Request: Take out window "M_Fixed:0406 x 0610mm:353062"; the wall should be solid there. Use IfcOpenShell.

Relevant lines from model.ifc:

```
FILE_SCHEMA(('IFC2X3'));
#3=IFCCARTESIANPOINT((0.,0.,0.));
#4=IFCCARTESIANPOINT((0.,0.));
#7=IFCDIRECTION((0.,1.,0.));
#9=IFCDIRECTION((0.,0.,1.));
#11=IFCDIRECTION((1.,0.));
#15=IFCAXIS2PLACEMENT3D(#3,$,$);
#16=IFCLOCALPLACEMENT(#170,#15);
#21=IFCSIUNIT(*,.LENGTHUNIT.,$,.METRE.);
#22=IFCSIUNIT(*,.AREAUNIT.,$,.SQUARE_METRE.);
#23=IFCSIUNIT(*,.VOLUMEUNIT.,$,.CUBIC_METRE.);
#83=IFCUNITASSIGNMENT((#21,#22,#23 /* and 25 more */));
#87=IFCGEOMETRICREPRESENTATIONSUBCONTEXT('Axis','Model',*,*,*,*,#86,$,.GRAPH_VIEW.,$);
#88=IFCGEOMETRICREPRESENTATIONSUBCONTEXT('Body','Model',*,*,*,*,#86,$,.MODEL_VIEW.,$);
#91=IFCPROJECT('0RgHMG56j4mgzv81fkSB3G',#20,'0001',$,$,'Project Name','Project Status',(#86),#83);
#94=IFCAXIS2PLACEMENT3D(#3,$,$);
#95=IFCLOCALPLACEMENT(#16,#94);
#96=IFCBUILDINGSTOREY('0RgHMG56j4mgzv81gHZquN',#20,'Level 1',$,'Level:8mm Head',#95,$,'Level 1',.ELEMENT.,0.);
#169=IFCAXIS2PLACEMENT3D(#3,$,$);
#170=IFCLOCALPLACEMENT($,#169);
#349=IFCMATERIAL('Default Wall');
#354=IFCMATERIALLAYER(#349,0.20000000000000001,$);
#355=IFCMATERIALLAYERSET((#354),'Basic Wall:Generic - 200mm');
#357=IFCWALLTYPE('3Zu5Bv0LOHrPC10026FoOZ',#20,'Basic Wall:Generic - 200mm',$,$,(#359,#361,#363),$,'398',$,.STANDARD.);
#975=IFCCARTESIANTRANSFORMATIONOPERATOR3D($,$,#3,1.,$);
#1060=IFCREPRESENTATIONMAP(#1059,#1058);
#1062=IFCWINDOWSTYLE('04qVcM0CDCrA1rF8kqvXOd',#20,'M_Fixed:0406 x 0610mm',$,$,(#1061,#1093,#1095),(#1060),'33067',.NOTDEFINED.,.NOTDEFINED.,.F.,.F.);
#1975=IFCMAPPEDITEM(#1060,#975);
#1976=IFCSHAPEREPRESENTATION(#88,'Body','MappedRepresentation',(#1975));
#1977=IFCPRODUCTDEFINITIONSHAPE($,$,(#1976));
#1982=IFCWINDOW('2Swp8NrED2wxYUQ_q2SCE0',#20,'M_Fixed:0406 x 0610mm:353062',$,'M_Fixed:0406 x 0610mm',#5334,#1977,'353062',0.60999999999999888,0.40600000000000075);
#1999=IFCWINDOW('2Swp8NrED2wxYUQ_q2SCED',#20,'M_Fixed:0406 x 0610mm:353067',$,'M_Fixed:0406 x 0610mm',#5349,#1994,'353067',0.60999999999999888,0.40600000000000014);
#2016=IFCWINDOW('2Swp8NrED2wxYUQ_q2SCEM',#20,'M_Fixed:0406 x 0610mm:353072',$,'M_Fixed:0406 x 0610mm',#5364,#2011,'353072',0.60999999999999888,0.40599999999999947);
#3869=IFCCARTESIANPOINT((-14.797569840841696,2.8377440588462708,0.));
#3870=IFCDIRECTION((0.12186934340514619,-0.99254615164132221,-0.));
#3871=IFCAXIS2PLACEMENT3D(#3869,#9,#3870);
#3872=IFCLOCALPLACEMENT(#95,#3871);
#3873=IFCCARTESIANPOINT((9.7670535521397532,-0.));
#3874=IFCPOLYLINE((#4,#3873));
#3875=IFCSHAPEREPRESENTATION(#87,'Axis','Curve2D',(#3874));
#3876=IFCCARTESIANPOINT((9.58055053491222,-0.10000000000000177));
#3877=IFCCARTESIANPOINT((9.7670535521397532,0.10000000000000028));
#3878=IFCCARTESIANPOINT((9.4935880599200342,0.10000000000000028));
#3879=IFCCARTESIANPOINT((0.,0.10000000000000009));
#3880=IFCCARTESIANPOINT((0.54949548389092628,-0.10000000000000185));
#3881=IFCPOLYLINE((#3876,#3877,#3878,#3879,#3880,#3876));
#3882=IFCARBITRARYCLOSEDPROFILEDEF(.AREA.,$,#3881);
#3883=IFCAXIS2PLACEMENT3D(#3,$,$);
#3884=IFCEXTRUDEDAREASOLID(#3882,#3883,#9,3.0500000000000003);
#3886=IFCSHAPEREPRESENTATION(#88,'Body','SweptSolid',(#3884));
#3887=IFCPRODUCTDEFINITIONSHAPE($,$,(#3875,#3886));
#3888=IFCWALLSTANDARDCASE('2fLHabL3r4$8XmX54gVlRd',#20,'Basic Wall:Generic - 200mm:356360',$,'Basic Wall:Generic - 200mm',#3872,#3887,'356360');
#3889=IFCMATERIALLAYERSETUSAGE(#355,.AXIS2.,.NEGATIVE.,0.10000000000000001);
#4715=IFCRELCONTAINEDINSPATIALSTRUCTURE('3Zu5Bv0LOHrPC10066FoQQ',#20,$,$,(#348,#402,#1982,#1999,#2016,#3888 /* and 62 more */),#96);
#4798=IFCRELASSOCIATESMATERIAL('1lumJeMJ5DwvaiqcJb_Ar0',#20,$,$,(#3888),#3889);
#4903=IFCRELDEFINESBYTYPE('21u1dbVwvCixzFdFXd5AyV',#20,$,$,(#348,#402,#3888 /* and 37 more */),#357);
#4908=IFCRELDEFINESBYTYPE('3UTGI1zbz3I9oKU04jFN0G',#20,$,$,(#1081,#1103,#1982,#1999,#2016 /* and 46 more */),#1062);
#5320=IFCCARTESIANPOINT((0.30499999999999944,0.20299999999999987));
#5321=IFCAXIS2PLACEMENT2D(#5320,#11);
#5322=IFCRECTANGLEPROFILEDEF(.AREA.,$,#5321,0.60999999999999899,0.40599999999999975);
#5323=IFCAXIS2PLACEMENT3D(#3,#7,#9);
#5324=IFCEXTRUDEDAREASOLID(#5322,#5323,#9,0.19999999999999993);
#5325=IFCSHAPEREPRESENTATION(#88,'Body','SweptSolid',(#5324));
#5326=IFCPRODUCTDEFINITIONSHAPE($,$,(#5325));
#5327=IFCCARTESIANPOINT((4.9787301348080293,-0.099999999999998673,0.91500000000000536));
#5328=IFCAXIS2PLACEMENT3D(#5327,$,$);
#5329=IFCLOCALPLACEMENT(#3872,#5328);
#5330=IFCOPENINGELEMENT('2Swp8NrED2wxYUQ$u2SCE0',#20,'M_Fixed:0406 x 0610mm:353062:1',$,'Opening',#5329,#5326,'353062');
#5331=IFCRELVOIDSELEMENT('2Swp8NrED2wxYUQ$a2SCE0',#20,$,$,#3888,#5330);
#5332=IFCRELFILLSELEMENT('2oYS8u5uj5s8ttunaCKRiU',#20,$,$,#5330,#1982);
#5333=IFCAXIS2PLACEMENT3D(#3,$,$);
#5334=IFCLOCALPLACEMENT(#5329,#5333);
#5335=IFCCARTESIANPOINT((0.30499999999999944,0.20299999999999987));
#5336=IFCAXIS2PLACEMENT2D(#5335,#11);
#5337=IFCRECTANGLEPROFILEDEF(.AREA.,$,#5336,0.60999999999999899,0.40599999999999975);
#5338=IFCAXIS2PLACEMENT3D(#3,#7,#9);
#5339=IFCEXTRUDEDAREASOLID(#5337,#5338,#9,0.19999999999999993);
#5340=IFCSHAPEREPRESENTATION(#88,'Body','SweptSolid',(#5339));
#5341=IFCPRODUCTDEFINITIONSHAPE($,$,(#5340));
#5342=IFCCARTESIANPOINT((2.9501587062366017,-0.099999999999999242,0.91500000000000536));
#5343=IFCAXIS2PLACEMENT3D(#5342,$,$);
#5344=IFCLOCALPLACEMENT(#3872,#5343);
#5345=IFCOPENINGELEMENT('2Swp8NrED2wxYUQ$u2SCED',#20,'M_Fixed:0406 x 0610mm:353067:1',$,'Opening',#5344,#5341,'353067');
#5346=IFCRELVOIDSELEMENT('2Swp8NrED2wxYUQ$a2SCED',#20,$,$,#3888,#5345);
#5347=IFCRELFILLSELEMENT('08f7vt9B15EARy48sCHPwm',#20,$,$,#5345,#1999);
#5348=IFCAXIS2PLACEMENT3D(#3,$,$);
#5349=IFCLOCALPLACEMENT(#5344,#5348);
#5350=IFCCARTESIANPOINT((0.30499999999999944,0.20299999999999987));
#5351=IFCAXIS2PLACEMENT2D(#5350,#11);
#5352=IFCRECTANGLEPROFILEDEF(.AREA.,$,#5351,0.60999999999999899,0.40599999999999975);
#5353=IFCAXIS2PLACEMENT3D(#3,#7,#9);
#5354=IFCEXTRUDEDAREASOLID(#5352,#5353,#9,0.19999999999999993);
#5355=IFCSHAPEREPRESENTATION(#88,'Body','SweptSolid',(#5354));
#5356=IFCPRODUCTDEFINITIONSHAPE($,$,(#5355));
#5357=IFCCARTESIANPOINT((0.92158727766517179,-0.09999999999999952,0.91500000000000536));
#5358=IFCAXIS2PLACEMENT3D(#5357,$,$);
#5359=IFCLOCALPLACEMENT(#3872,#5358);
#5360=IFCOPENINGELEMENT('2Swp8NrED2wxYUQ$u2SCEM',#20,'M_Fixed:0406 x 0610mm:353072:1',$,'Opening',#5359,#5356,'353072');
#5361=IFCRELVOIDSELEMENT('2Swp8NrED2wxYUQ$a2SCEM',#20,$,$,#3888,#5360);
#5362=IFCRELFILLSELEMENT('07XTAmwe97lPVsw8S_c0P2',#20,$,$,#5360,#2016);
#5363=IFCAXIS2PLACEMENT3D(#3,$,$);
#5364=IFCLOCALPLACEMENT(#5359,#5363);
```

```python
import ifcopenshell
import ifcopenshell.api.feature
import ifcopenshell.api.root
import ifcopenshell.geom
import ifcopenshell.util.shape

model = ifcopenshell.open("model.ifc")
settings = ifcopenshell.geom.settings()


def volume(element):
    """Net volume in cubic metres, openings subtracted."""
    shape = ifcopenshell.geom.create_shape(settings, element)
    return ifcopenshell.util.shape.get_volume(shape.geometry)


window = model.by_id(1982)
opening = window.FillsVoids[0].RelatingOpeningElement
wall = opening.VoidsElements[0].RelatingBuildingElement
before = volume(wall)

ifcopenshell.api.root.remove_product(model, product=window)
ifcopenshell.api.feature.remove_feature(model, feature=opening)

after = volume(wall)

print(f"wall volume {before:.3f} -> {after:.3f} m3")

model.write("model_edited.ifc")
```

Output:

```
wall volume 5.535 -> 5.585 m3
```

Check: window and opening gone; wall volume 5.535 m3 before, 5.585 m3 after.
